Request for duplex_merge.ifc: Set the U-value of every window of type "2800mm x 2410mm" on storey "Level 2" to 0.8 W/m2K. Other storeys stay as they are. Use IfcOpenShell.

First a look at what the model holds.

```python
import ifcopenshell
import ifcopenshell.util.element

model = ifcopenshell.open("duplex_merge.ifc")
print(model.schema)
storey = next(s for s in model.by_type("IfcBuildingStorey") if s.Name == "Level 2")
windows = [e for e in ifcopenshell.util.element.get_decomposition(storey) if e.is_a("IfcWindow")]
seen = {}
for e in windows:
    element_type = ifcopenshell.util.element.get_type(e)
    key = (element_type.Name if element_type != e and element_type else None, ifcopenshell.util.element.get_pset(e, "Pset_WindowCommon", "ThermalTransmittance"))
    seen[key] = seen.get(key, 0) + 1
for (name, value), count in sorted(seen.items(), key=str):
    print(count, "x", name, "|", value)
```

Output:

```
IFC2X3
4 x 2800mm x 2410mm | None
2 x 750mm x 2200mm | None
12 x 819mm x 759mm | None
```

```python
import ifcopenshell
import ifcopenshell.api.pset
import ifcopenshell.util.element

model = ifcopenshell.open("duplex_merge.ifc")

storey = next(s for s in model.by_type("IfcBuildingStorey") if s.Name == "Level 2")
windows = [e for e in ifcopenshell.util.element.get_decomposition(storey) if e.is_a("IfcWindow")]

count = 0
for e in windows:
    element_type = ifcopenshell.util.element.get_type(e)
    if element_type in (None, e) or element_type.Name != "2800mm x 2410mm":
        continue
    # add_pset returns the element's existing set when there is one.
    pset = ifcopenshell.api.pset.add_pset(model, product=e, name="Pset_WindowCommon")
    ifcopenshell.api.pset.edit_pset(model, pset=pset, properties={"ThermalTransmittance": 0.8})
    count += 1

print(count, "windows updated")

model.write("duplex_merge_updated.ifc")
```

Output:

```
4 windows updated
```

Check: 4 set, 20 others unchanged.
